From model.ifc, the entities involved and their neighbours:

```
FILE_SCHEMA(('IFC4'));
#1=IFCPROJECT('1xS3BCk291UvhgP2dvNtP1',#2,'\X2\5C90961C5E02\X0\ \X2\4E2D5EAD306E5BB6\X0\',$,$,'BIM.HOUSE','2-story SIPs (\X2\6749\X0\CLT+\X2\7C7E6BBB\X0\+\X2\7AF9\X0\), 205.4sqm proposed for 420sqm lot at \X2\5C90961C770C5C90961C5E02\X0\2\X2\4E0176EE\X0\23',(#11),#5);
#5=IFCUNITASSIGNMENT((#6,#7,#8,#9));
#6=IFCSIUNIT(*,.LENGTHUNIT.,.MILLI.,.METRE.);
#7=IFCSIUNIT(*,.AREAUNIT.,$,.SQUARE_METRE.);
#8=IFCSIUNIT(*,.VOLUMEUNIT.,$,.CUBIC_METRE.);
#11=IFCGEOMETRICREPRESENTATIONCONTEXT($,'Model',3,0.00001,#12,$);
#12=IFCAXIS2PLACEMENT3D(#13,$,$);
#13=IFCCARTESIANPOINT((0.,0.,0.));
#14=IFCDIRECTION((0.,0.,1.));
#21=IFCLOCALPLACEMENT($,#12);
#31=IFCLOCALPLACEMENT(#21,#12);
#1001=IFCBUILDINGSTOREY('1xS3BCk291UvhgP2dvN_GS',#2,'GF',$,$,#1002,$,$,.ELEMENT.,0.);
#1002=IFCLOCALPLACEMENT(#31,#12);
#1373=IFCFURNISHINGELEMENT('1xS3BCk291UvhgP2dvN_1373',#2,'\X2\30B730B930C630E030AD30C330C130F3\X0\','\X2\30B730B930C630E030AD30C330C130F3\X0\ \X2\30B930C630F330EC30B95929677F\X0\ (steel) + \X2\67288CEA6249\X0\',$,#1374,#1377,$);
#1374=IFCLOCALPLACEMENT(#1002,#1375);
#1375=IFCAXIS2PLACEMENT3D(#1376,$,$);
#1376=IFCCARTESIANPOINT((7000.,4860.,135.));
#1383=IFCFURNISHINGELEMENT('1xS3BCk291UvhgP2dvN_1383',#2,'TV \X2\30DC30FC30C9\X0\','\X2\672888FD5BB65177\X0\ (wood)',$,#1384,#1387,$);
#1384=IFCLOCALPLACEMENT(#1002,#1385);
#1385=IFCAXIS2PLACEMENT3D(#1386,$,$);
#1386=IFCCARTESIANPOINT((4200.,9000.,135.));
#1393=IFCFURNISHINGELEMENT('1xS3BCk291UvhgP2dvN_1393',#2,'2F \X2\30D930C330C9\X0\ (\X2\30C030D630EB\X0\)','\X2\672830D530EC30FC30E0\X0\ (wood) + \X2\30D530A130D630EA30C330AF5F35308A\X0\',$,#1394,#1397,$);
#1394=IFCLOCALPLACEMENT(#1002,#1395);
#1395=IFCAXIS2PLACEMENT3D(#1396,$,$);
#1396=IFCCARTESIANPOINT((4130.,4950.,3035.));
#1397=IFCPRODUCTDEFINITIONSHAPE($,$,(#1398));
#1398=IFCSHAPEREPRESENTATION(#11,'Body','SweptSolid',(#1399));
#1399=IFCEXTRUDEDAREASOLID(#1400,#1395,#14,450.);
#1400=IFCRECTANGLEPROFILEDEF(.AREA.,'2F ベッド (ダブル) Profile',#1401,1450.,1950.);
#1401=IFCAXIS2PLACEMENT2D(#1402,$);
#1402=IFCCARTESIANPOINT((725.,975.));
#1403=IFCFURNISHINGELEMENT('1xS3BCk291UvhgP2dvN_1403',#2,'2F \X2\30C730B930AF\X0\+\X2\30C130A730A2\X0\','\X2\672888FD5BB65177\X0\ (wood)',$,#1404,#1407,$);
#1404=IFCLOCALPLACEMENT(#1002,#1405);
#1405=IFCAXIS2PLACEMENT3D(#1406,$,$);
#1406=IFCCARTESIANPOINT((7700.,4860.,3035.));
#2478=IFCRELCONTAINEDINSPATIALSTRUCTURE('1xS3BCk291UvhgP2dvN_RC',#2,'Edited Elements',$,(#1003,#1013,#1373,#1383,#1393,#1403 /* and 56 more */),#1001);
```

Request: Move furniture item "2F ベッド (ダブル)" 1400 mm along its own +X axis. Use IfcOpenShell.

```python
import ifcopenshell
import ifcopenshell.api.geometry
import ifcopenshell.util.placement
import ifcopenshell.util.unit

model = ifcopenshell.open("model.ifc")
unit_scale = ifcopenshell.util.unit.calculate_unit_scale(model)

item = model.by_guid("1xS3BCk291UvhgP2dvN_1393")
matrix = ifcopenshell.util.placement.get_local_placement(item.ObjectPlacement)
matrix[:3, 3] += matrix[:3, 0] * 1.4 / unit_scale
ifcopenshell.api.geometry.edit_object_placement(model, product=item, matrix=matrix, is_si=False)

print(ifcopenshell.util.placement.get_local_placement(item.ObjectPlacement).round(3) + 0.0)

model.write("model_updated.ifc")
```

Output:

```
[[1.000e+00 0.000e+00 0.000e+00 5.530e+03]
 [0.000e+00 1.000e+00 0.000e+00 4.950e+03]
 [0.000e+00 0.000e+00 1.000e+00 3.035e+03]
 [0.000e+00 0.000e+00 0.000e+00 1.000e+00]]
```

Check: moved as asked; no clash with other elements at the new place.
